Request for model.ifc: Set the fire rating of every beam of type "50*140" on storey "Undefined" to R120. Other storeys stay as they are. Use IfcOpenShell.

First a look at what the model holds.

```python
import ifcopenshell
import ifcopenshell.util.element

model = ifcopenshell.open("model.ifc")
print(model.schema)
storey = next(s for s in model.by_type("IfcBuildingStorey") if s.Name == "Undefined")
beams = [e for e in ifcopenshell.util.element.get_decomposition(storey) if e.is_a("IfcBeam")]
seen = {}
for e in beams:
    element_type = ifcopenshell.util.element.get_type(e)
    key = (element_type.Name if element_type != e and element_type else None, ifcopenshell.util.element.get_pset(e, "Pset_BeamCommon", "FireRating"))
    seen[key] = seen.get(key, 0) + 1
for (name, value), count in sorted(seen.items(), key=str):
    print(count, "x", name, "|", value)
```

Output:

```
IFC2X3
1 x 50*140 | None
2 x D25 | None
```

```python
import ifcopenshell
import ifcopenshell.api.pset
import ifcopenshell.util.element

model = ifcopenshell.open("model.ifc")

storey = next(s for s in model.by_type("IfcBuildingStorey") if s.Name == "Undefined")
beams = [e for e in ifcopenshell.util.element.get_decomposition(storey) if e.is_a("IfcBeam")]

count = 0
for e in beams:
    element_type = ifcopenshell.util.element.get_type(e)
    if element_type in (None, e) or element_type.Name != "50*140":
        continue
    # add_pset returns the element's existing set when there is one.
    pset = ifcopenshell.api.pset.add_pset(model, product=e, name="Pset_BeamCommon")
    ifcopenshell.api.pset.edit_pset(model, pset=pset, properties={"FireRating": "R120"})
    count += 1

print(count, "beams updated")

model.write("model_edited.ifc")
```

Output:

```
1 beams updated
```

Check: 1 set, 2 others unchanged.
